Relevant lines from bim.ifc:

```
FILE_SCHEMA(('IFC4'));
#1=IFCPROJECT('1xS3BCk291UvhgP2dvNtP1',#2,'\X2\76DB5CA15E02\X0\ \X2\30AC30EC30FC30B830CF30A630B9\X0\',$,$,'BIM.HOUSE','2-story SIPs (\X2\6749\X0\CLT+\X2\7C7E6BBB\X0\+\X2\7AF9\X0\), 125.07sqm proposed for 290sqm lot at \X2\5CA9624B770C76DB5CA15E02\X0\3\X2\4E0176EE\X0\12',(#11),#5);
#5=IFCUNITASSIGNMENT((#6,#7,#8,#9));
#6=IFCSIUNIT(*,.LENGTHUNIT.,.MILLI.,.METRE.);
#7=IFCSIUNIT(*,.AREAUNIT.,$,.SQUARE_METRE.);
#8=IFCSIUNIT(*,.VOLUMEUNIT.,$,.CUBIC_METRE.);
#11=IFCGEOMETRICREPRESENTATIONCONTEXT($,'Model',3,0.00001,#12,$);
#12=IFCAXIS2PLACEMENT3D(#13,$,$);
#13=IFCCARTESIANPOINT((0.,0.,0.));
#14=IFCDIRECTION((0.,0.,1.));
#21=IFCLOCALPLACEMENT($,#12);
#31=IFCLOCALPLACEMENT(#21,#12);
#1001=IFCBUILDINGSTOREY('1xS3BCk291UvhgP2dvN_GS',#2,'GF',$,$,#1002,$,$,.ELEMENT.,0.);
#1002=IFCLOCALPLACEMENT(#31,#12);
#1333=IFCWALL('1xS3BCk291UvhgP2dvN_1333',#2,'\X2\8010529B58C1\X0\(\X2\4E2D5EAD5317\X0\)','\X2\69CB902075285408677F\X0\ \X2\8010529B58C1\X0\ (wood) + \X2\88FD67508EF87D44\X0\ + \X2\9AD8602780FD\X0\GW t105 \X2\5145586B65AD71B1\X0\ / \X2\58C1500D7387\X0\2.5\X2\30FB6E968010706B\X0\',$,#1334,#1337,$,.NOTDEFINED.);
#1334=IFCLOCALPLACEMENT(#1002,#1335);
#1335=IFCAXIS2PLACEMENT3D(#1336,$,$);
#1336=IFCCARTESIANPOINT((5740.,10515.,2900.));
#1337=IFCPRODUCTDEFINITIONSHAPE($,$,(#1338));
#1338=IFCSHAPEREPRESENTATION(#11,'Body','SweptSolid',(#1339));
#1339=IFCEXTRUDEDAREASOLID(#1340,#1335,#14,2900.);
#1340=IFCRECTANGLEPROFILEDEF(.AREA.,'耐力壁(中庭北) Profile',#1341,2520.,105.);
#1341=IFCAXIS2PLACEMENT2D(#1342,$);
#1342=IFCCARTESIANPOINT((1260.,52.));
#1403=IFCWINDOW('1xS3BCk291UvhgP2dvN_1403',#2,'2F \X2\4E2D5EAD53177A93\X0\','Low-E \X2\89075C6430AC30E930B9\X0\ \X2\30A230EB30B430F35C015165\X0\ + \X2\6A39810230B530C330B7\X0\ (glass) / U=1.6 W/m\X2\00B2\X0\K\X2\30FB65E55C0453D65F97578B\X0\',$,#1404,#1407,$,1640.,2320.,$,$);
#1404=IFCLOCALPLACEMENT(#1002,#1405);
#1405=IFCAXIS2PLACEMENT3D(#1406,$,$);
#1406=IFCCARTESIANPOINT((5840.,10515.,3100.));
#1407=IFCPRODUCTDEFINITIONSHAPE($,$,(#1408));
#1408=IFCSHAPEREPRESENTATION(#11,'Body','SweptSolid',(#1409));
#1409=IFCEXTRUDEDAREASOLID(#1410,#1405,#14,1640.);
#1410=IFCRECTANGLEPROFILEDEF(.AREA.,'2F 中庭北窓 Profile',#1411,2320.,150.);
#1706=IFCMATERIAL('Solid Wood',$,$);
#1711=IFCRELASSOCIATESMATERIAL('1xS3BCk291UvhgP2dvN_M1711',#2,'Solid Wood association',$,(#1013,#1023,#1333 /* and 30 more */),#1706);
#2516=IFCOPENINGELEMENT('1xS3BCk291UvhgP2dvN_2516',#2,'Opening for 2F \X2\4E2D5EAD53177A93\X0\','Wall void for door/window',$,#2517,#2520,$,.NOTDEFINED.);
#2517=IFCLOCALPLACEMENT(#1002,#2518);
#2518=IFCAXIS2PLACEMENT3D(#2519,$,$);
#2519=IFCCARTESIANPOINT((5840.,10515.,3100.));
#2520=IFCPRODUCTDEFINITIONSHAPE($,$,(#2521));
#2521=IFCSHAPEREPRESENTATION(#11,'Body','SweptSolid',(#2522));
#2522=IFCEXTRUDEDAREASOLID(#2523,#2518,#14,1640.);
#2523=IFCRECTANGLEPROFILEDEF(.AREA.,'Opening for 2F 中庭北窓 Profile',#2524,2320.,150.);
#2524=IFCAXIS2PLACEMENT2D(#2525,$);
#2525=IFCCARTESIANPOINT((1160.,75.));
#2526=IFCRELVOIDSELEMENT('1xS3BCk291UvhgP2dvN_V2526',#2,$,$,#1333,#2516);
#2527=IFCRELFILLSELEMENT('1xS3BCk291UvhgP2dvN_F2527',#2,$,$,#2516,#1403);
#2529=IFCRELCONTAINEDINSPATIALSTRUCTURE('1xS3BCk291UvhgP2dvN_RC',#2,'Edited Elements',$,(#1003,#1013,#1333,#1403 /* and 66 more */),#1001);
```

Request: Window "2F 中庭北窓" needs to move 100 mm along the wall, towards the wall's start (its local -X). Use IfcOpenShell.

```python
import ifcopenshell
import ifcopenshell.api.geometry
import ifcopenshell.util.placement
import ifcopenshell.util.unit

model = ifcopenshell.open("bim.ifc")
unit_scale = ifcopenshell.util.unit.calculate_unit_scale(model)

window = model.by_guid("1xS3BCk291UvhgP2dvN_1403")
opening = window.FillsVoids[0].RelatingOpeningElement
wall = opening.VoidsElements[0].RelatingBuildingElement

wall_matrix = ifcopenshell.util.placement.get_local_placement(wall.ObjectPlacement)
shift = wall_matrix[:3, 0] * -0.1 / unit_scale
before = ifcopenshell.util.placement.get_local_placement(window.ObjectPlacement)[:3, 3].copy()

# The window is not placed relative to its opening, so move both.
for product in (opening, window):
    matrix = ifcopenshell.util.placement.get_local_placement(product.ObjectPlacement)
    matrix[:3, 3] += shift
    ifcopenshell.api.geometry.edit_object_placement(model, product=product, matrix=matrix, is_si=False)

after = ifcopenshell.util.placement.get_local_placement(window.ObjectPlacement)[:3, 3]
print("window moved by", (after - before).round(3) + 0.0)

model.write("bim_edited.ifc")
```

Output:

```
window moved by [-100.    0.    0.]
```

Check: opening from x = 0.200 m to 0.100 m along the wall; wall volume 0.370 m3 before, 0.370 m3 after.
